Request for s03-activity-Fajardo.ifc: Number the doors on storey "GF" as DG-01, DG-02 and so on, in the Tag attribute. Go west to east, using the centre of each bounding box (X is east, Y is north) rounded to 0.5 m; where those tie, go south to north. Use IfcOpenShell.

First a look at what the model holds.

```python
import ifcopenshell
import ifcopenshell.util.element
import ifcopenshell.util.placement

model = ifcopenshell.open("s03-activity-Fajardo.ifc")
print(model.schema)
storey = next(s for s in model.by_type("IfcBuildingStorey") if s.Name == "GF")
doors = [e for e in ifcopenshell.util.element.get_decomposition(storey) if e.is_a("IfcDoor")]
for e in sorted(doors, key=lambda e: e.id()):
    origin = ifcopenshell.util.placement.get_local_placement(e.ObjectPlacement)[:3, 3]
    print(e.id(), e.Tag, e.Name, origin.round(2) + 0.0, sep=" | ")
```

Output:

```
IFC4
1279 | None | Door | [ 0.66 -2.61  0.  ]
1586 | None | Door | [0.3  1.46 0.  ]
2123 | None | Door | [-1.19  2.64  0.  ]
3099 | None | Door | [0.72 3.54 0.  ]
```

```python
import ifcopenshell
import ifcopenshell.geom
import ifcopenshell.util.element
import ifcopenshell.util.shape

model = ifcopenshell.open("s03-activity-Fajardo.ifc")
settings = ifcopenshell.geom.settings()
settings.set("use-world-coords", True)


def centre(element):
    shape = ifcopenshell.geom.create_shape(settings, element)
    return ifcopenshell.util.shape.get_bbox_centroid(shape.geometry)


storey = next(s for s in model.by_type("IfcBuildingStorey") if s.Name == "GF")
doors = [e for e in ifcopenshell.util.element.get_decomposition(storey) if e.is_a("IfcDoor")]

# Insertion points can sit at a corner or the storey origin, so sort by the geometry (in metres).
centres = {e: centre(e) for e in doors}
doors.sort(key=lambda e: (round(centres[e][0] / 0.5), centres[e][1]))

for i, e in enumerate(doors, start=1):
    number = f"DG-{i:02d}"
    e.Tag = number
    print(e.id(), number)

model.write("s03-activity-Fajardo_edited.ifc")
```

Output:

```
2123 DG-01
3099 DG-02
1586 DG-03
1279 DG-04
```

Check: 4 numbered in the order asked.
